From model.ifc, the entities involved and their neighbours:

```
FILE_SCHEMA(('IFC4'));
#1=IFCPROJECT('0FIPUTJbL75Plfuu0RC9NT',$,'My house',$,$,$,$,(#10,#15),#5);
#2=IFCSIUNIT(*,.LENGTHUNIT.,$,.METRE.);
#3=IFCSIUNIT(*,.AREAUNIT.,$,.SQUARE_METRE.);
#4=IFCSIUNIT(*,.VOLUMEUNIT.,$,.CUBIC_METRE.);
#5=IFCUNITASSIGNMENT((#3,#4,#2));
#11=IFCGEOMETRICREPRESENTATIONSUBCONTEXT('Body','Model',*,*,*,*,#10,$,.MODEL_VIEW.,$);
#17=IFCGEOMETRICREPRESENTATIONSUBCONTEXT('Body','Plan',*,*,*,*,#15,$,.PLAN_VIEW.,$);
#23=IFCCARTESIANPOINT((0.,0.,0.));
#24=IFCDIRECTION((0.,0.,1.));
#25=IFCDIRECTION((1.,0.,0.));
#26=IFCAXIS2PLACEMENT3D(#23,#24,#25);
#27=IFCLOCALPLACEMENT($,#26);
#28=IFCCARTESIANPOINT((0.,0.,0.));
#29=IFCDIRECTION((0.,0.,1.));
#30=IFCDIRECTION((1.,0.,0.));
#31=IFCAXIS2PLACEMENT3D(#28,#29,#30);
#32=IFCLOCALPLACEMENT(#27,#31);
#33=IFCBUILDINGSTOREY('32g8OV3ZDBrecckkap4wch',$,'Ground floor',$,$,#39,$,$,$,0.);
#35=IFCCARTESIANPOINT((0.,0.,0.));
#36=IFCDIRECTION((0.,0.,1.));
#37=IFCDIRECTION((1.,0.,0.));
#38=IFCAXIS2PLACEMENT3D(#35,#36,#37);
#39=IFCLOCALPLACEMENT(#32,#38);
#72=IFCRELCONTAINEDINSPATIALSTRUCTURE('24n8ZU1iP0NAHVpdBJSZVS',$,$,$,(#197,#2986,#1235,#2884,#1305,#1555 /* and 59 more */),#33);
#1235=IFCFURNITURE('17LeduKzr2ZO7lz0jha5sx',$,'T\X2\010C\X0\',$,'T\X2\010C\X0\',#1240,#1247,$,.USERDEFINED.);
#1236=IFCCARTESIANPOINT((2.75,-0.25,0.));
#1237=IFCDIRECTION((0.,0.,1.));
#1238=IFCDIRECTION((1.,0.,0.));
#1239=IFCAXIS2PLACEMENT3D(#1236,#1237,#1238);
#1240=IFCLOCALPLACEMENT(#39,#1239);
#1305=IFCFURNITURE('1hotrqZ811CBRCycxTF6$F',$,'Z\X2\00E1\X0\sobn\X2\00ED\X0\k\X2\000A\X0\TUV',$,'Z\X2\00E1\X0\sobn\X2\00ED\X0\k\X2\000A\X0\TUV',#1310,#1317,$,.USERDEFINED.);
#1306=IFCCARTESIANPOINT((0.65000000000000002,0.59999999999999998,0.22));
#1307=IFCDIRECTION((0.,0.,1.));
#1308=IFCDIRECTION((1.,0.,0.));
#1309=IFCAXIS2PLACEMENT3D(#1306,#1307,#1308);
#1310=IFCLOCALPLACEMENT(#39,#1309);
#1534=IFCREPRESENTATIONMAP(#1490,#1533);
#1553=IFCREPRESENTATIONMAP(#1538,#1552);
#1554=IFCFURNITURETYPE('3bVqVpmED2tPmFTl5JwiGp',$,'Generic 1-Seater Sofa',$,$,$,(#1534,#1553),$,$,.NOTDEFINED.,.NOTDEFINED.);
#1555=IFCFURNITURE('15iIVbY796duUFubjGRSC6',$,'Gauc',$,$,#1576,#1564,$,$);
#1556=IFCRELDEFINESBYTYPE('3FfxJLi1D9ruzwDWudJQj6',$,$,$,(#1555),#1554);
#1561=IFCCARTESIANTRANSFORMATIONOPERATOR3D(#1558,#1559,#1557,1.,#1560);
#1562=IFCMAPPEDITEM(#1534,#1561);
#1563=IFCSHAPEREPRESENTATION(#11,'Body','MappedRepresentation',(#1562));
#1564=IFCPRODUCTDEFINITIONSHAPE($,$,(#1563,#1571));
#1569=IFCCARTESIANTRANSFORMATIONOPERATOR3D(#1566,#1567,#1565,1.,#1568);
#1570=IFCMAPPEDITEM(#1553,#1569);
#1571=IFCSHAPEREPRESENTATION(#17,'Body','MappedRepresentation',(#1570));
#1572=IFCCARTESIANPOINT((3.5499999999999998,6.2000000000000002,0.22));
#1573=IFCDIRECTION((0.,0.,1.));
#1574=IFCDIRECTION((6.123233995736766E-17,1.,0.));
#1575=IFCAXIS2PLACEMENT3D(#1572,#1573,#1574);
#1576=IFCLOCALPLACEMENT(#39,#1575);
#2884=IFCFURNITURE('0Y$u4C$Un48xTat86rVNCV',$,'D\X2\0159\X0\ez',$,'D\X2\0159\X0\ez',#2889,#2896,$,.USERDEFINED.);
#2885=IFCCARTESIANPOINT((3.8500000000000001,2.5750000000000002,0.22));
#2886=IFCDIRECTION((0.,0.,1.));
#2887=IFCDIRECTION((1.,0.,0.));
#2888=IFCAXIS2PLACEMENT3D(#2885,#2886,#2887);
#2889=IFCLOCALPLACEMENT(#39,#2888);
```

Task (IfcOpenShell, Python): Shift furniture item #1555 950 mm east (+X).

```python
import ifcopenshell
import ifcopenshell.api.geometry
import ifcopenshell.util.placement
import ifcopenshell.util.unit

model = ifcopenshell.open("model.ifc")
unit_scale = ifcopenshell.util.unit.calculate_unit_scale(model)

item = model.by_guid("15iIVbY796duUFubjGRSC6")
matrix = ifcopenshell.util.placement.get_local_placement(item.ObjectPlacement)
matrix[0, 3] += 0.95 / unit_scale
ifcopenshell.api.geometry.edit_object_placement(model, product=item, matrix=matrix, is_si=False)

print(ifcopenshell.util.placement.get_local_placement(item.ObjectPlacement).round(3) + 0.0)

model.write("model_v2.ifc")
```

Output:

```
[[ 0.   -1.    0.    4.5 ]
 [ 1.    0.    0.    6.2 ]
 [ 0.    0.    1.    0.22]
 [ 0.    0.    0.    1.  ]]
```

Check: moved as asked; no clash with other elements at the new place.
